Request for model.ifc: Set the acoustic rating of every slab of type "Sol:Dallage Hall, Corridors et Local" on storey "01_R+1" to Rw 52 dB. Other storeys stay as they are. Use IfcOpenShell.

First a look at what the model holds.

```python
import ifcopenshell
import ifcopenshell.util.element

model = ifcopenshell.open("model.ifc")
print(model.schema)
storey = next(s for s in model.by_type("IfcBuildingStorey") if s.Name == "01_R+1")
slabs = [e for e in ifcopenshell.util.element.get_decomposition(storey) if e.is_a("IfcSlab")]
seen = {}
for e in slabs:
    element_type = ifcopenshell.util.element.get_type(e)
    key = (element_type.Name if element_type != e and element_type else None, ifcopenshell.util.element.get_pset(e, "Pset_SlabCommon", "AcousticRating"))
    seen[key] = seen.get(key, 0) + 1
for (name, value), count in sorted(seen.items(), key=str):
    print(count, "x", name, "|", value)
```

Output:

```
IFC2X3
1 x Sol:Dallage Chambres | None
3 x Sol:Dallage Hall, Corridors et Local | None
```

```python
import ifcopenshell
import ifcopenshell.api.pset
import ifcopenshell.util.element

model = ifcopenshell.open("model.ifc")

storey = next(s for s in model.by_type("IfcBuildingStorey") if s.Name == "01_R+1")
slabs = [e for e in ifcopenshell.util.element.get_decomposition(storey) if e.is_a("IfcSlab")]

count = 0
for e in slabs:
    element_type = ifcopenshell.util.element.get_type(e)
    if element_type in (None, e) or element_type.Name != "Sol:Dallage Hall, Corridors et Local":
        continue
    # add_pset returns the element's existing set when there is one.
    pset = ifcopenshell.api.pset.add_pset(model, product=e, name="Pset_SlabCommon")
    ifcopenshell.api.pset.edit_pset(model, pset=pset, properties={"AcousticRating": "Rw 52 dB"})
    count += 1

print(count, "slabs updated")

model.write("model-out.ifc")
```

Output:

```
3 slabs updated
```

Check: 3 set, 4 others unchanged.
